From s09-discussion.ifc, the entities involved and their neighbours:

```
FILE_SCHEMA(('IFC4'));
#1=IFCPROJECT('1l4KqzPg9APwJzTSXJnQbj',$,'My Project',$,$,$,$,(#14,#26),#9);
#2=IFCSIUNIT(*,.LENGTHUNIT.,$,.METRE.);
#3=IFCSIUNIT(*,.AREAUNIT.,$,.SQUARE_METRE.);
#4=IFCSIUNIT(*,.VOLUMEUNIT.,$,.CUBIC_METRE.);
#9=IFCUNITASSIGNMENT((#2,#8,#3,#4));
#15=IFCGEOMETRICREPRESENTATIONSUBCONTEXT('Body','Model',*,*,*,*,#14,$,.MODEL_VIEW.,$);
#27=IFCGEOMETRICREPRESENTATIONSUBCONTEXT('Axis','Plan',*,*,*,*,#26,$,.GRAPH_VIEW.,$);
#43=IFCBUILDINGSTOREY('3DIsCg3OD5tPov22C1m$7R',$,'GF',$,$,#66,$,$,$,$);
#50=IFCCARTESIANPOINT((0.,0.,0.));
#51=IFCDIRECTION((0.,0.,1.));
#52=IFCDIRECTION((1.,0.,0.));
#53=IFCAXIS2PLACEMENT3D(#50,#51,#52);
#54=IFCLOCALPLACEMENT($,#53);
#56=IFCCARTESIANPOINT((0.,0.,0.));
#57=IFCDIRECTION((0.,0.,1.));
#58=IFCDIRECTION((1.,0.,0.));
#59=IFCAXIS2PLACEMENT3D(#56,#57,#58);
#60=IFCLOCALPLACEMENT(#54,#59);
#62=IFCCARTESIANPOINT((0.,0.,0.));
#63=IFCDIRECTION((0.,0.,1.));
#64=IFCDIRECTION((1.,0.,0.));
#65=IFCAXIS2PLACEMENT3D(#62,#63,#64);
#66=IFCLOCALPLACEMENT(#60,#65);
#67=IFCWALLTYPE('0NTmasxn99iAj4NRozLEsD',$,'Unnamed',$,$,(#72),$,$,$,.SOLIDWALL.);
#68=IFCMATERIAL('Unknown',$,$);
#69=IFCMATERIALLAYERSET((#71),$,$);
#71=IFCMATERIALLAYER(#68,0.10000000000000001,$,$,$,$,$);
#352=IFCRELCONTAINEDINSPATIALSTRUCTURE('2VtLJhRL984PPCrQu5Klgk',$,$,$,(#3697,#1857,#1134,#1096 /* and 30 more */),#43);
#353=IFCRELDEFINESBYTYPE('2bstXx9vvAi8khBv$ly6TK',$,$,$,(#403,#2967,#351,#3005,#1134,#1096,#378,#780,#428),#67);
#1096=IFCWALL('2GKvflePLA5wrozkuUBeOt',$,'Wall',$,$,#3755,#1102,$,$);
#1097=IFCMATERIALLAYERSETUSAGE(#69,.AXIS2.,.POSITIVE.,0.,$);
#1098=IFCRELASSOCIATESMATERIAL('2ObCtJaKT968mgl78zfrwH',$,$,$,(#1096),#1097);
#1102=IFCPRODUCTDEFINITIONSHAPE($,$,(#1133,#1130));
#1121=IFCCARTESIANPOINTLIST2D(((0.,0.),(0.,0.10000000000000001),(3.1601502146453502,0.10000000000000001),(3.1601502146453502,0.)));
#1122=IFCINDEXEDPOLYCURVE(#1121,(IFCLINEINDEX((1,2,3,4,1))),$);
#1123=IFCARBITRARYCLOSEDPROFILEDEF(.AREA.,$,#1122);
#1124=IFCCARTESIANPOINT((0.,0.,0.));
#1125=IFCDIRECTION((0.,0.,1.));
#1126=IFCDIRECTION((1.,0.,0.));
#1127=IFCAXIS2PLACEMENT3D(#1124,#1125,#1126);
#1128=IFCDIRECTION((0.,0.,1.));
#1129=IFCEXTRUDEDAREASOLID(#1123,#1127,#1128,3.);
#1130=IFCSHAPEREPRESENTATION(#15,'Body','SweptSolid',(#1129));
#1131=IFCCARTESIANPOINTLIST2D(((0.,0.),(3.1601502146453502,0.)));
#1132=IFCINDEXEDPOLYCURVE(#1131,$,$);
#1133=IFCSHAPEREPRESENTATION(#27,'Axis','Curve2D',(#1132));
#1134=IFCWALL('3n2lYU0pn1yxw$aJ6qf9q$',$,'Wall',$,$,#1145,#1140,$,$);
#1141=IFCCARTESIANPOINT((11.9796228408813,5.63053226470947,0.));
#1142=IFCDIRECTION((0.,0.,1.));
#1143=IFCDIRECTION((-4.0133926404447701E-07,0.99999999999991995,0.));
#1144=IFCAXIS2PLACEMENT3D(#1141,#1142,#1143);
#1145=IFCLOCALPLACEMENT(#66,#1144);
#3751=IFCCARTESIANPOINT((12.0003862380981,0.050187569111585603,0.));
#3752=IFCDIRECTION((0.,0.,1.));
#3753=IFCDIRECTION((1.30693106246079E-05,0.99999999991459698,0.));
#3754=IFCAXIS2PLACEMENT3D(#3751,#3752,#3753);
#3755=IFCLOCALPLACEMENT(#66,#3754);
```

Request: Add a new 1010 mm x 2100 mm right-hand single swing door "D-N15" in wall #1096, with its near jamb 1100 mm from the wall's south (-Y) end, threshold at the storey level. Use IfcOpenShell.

```python
import numpy as np
import ifcopenshell
import ifcopenshell.api.feature
import ifcopenshell.api.geometry
import ifcopenshell.api.root
import ifcopenshell.api.spatial
import ifcopenshell.geom
import ifcopenshell.util.element
import ifcopenshell.util.placement
import ifcopenshell.util.representation
import ifcopenshell.util.shape
import ifcopenshell.util.unit

model = ifcopenshell.open("s09-discussion.ifc")
unit_scale = ifcopenshell.util.unit.calculate_unit_scale(model)
settings = ifcopenshell.geom.settings()


def volume(element):
    """Net volume in cubic metres, openings subtracted."""
    shape = ifcopenshell.geom.create_shape(settings, element)
    return ifcopenshell.util.shape.get_volume(shape.geometry)


wall = model.by_guid("2GKvflePLA5wrozkuUBeOt")
storey = ifcopenshell.util.element.get_container(wall, ifc_class="IfcBuildingStorey")
context = ifcopenshell.util.representation.get_context(model, "Model", "Body", "MODEL_VIEW")
before = volume(wall)

width, height, from_end, sill = 1.01, 2.1, 1.1, 0.0  # metres

# The wall runs along its own X axis, and the end named is its -X end.
wall_shape = ifcopenshell.geom.create_shape(settings, wall)
x, y, z = ifcopenshell.util.shape.get_vertices(wall_shape.geometry).T
start = x.min() + from_end
face, thickness = float(y.min()), float(y.max() - y.min())
wall_matrix = ifcopenshell.util.placement.get_local_placement(wall.ObjectPlacement)
level = ifcopenshell.util.placement.get_local_placement(storey.ObjectPlacement)[2, 3]


def in_wall(x, y):
    """Placement at x, y metres in the wall's axes, at sill height."""
    matrix = wall_matrix.copy()
    matrix[:, 3] = wall_matrix @ np.array([x / unit_scale, y / unit_scale, 0.0, 1.0])
    matrix[2, 3] = level + sill / unit_scale
    return matrix


# Opening: a box that overshoots both wall faces by 50 mm.
opening = ifcopenshell.api.root.create_entity(model, ifc_class="IfcOpeningElement", predefined_type="OPENING")
box = ifcopenshell.api.geometry.add_wall_representation(
    model, context=context, length=width, height=height, thickness=thickness + 0.1
)
ifcopenshell.api.geometry.assign_representation(model, product=opening, representation=box)
ifcopenshell.api.geometry.edit_object_placement(model, product=opening, matrix=in_wall(start, face - 0.05), is_si=False)
ifcopenshell.api.feature.add_feature(model, feature=opening, element=wall)

door = ifcopenshell.api.root.create_entity(model, ifc_class="IfcDoor", name="D-N15", predefined_type="DOOR")
door.OverallWidth, door.OverallHeight = width / unit_scale, height / unit_scale
door.OperationType = "SINGLE_SWING_RIGHT"
body = ifcopenshell.api.geometry.add_door_representation(
    model,
    context=context,
    overall_width=door.OverallWidth,
    overall_height=door.OverallHeight,
    operation_type="SINGLE_SWING_RIGHT",
    lining_properties={"LiningDepth": thickness / unit_scale, "ThresholdDepth": thickness / unit_scale},
)
ifcopenshell.api.geometry.assign_representation(model, product=door, representation=body)
ifcopenshell.api.spatial.assign_container(model, products=[door], relating_structure=storey)
ifcopenshell.api.feature.add_filling(model, opening=opening, element=door)

# The lining spans the wall, so the door starts at the wall face.
ifcopenshell.api.geometry.edit_object_placement(model, product=door, matrix=in_wall(start, face), is_si=False)

after = volume(wall)

print(f"wall volume {before:.3f} -> {after:.3f} m3")

model.write("s09-discussion_edited.ifc")
```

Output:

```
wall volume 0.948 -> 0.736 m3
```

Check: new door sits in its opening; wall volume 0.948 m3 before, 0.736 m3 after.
